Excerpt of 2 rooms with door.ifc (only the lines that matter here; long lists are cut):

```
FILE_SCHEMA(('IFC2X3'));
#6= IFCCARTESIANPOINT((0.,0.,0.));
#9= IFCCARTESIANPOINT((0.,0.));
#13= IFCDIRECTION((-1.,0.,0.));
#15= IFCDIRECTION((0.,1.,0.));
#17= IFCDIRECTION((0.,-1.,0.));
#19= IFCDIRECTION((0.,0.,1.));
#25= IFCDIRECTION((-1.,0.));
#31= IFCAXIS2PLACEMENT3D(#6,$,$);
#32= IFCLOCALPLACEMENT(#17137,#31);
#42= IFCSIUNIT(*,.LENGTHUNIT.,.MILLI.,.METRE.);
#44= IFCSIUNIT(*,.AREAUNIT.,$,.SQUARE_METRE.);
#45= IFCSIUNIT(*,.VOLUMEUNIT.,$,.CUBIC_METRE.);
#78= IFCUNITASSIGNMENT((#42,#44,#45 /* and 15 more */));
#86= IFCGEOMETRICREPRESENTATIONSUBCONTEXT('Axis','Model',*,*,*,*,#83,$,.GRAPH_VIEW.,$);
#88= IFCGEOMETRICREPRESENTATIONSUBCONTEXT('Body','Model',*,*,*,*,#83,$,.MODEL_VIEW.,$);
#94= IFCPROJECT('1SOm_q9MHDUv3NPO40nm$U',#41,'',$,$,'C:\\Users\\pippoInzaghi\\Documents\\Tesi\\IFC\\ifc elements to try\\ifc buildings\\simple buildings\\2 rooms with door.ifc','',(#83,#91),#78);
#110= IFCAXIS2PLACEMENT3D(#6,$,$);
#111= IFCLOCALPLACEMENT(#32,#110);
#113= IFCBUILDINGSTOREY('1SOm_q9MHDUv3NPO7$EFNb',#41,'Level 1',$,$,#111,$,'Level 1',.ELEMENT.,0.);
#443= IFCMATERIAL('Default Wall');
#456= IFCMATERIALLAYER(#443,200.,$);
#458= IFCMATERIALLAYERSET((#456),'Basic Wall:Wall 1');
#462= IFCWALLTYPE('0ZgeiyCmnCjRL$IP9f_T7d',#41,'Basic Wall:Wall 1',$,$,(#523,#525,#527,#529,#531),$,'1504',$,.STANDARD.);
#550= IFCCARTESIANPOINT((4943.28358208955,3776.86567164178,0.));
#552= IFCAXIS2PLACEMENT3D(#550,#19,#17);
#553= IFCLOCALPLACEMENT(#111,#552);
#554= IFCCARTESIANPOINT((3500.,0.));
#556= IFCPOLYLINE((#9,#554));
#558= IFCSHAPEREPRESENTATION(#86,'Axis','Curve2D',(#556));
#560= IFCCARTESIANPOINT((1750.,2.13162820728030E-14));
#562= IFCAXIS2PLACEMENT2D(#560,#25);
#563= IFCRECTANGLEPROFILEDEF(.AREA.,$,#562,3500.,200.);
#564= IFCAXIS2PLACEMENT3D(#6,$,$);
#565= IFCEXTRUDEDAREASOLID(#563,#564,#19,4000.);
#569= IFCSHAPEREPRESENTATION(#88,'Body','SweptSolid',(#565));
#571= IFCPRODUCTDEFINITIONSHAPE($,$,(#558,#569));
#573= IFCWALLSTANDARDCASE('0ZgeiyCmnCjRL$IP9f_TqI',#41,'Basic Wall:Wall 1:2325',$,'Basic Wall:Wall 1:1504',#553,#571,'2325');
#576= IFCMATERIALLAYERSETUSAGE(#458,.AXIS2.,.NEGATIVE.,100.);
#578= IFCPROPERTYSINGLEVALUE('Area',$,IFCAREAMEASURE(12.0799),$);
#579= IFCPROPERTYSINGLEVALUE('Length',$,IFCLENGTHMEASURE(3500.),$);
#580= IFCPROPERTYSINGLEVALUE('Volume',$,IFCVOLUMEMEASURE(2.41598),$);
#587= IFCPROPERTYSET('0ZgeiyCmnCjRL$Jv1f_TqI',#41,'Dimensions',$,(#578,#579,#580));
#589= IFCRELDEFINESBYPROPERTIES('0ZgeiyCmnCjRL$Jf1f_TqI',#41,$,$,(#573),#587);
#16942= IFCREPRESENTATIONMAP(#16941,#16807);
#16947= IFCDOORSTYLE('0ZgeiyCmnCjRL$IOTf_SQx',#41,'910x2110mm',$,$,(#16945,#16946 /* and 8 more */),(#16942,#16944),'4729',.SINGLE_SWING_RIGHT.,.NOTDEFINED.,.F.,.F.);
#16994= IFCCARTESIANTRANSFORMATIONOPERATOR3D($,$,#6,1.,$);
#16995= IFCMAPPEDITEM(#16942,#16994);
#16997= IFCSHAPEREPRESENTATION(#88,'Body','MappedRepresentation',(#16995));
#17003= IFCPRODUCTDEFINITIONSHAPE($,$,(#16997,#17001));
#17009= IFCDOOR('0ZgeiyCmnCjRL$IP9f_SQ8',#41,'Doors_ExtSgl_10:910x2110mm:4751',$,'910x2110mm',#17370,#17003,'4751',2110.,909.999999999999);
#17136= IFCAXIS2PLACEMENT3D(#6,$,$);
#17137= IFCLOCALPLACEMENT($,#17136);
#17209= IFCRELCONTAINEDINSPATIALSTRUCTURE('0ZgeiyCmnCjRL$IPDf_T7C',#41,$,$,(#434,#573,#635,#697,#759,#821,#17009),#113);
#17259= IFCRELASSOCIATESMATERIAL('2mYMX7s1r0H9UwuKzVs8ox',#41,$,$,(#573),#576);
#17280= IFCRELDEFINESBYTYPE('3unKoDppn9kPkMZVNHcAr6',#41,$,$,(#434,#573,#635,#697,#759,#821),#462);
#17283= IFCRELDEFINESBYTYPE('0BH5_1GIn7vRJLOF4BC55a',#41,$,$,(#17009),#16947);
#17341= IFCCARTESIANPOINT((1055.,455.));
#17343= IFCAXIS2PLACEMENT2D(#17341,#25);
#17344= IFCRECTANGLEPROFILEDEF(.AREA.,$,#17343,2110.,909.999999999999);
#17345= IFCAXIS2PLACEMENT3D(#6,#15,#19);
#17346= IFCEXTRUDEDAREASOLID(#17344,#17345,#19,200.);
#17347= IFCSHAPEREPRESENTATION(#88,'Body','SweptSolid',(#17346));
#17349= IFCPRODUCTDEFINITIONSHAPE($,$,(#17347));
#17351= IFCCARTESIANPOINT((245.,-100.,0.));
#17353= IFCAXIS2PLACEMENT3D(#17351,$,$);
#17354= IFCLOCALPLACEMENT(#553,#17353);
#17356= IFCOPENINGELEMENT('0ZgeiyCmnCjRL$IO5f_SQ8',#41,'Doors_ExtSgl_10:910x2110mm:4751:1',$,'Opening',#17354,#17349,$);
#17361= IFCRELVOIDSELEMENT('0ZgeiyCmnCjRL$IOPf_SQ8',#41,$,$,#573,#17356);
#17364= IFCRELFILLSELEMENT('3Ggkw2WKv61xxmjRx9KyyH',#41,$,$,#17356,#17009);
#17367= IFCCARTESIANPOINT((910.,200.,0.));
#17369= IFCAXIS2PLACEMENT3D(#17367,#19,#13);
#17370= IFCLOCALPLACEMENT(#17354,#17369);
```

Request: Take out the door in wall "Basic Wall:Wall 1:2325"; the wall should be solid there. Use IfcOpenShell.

```python
import ifcopenshell
import ifcopenshell.api.feature
import ifcopenshell.api.pset
import ifcopenshell.api.root
import ifcopenshell.geom
import ifcopenshell.util.element
import ifcopenshell.util.shape
import ifcopenshell.util.unit

model = ifcopenshell.open("2 rooms with door.ifc")
area_scale = ifcopenshell.util.unit.calculate_unit_scale(model, "AREAUNIT")
volume_scale = ifcopenshell.util.unit.calculate_unit_scale(model, "VOLUMEUNIT")
settings = ifcopenshell.geom.settings()


def volume(element):
    """Net volume in cubic metres, openings subtracted."""
    shape = ifcopenshell.geom.create_shape(settings, element)
    return ifcopenshell.util.shape.get_volume(shape.geometry)


door = model.by_guid("0ZgeiyCmnCjRL$IP9f_SQ8")
opening = door.FillsVoids[0].RelatingOpeningElement
wall = opening.VoidsElements[0].RelatingBuildingElement
before = volume(wall)

ifcopenshell.api.root.remove_product(model, product=door)
ifcopenshell.api.feature.remove_feature(model, feature=opening)

after = volume(wall)
thickness = 0.2  # wall thickness in metres

# Update the wall's stored quantities.
pset = model.by_id(ifcopenshell.util.element.get_pset(wall, "Dimensions", should_inherit=False)["id"])
ifcopenshell.api.pset.edit_pset(model, pset=pset, properties={
    "Area": model.create_entity("IfcAreaMeasure", after / thickness / area_scale),
    "Volume": model.create_entity("IfcVolumeMeasure", after / volume_scale),
})

print(f"wall volume {before:.3f} -> {after:.3f} m3")

model.write("2 rooms with door-out.ifc")
```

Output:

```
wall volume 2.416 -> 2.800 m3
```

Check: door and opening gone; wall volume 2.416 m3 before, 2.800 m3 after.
